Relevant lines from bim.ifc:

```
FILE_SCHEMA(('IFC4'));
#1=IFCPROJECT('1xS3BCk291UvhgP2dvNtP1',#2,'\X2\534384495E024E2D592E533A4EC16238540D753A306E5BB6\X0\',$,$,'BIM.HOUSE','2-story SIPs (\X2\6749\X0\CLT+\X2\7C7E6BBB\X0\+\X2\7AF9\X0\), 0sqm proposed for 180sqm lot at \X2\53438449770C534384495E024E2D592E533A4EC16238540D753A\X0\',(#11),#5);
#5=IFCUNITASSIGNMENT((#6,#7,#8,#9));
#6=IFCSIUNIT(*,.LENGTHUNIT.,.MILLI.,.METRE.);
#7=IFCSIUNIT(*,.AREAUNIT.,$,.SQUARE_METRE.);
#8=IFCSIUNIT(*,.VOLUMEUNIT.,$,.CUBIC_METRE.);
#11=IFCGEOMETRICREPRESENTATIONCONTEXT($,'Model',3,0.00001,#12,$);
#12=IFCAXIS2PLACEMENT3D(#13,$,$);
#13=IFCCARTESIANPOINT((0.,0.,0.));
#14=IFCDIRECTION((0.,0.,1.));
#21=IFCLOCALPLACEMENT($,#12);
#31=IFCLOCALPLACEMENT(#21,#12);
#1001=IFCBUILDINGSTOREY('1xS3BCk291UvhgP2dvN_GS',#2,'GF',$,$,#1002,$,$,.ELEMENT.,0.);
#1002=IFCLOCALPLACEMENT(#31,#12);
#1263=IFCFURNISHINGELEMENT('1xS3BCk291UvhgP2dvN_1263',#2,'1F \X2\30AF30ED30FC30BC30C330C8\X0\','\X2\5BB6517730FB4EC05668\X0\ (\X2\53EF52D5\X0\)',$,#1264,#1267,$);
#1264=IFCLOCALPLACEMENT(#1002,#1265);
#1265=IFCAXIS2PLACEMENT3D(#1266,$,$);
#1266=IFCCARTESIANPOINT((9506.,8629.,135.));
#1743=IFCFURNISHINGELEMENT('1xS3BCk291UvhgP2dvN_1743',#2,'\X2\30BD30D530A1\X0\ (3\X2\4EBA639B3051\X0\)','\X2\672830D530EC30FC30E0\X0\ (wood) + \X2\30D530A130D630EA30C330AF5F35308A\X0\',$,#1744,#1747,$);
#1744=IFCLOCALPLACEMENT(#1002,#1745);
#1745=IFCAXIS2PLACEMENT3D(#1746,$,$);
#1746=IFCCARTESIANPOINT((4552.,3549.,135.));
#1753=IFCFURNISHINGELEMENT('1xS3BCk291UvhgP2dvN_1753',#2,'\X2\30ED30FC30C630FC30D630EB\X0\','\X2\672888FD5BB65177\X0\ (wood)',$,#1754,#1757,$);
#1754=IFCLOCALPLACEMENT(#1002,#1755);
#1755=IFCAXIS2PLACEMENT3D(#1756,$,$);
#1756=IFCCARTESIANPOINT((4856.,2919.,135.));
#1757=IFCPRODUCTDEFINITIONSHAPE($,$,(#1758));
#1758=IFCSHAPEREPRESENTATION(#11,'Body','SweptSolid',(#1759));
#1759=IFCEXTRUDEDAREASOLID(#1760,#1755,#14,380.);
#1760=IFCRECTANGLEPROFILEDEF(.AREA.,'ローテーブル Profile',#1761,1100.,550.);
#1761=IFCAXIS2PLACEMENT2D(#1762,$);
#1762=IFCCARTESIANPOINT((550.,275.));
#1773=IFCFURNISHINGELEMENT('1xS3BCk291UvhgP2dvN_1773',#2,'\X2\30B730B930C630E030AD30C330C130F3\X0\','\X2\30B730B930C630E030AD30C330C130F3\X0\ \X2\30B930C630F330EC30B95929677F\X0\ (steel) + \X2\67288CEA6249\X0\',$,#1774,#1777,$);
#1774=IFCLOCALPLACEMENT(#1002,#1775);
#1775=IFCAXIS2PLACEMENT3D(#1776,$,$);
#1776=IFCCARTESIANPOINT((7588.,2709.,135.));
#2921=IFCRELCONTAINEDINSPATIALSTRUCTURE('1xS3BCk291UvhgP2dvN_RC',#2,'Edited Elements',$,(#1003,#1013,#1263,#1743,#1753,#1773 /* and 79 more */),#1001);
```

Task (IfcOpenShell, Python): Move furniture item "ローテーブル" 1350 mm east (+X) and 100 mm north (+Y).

```python
import ifcopenshell
import ifcopenshell.api.geometry
import ifcopenshell.util.placement
import ifcopenshell.util.unit

model = ifcopenshell.open("bim.ifc")
unit_scale = ifcopenshell.util.unit.calculate_unit_scale(model)

item = model.by_guid("1xS3BCk291UvhgP2dvN_1753")
matrix = ifcopenshell.util.placement.get_local_placement(item.ObjectPlacement)
matrix[0, 3] += 1.35 / unit_scale
matrix[1, 3] += 0.1 / unit_scale
ifcopenshell.api.geometry.edit_object_placement(model, product=item, matrix=matrix, is_si=False)

print(ifcopenshell.util.placement.get_local_placement(item.ObjectPlacement).round(3) + 0.0)

model.write("bim_updated.ifc")
```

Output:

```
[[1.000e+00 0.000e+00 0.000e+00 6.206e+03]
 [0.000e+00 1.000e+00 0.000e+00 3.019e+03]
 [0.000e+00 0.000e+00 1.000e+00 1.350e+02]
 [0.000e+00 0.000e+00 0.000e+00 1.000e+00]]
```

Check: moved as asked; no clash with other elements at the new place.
